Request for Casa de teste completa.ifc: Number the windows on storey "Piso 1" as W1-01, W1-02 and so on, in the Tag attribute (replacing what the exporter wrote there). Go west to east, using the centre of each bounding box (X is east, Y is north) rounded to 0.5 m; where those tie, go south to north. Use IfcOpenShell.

First a look at what the model holds.

```python
import ifcopenshell
import ifcopenshell.util.element
import ifcopenshell.util.placement

model = ifcopenshell.open("Casa de teste completa.ifc")
print(model.schema)
storey = next(s for s in model.by_type("IfcBuildingStorey") if s.Name == "Piso 1")
windows = [e for e in ifcopenshell.util.element.get_decomposition(storey) if e.is_a("IfcWindow")]
for e in sorted(windows, key=lambda e: e.id()):
    origin = ifcopenshell.util.placement.get_local_placement(e.ObjectPlacement)[:3, 3]
    print(e.id(), e.Tag, e.Name, origin.round(2) + 0.0, sep=" | ")
```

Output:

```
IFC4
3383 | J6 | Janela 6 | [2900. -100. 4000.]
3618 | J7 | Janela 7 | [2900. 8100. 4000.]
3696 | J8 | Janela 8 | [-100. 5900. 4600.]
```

```python
import ifcopenshell
import ifcopenshell.geom
import ifcopenshell.util.element
import ifcopenshell.util.shape

model = ifcopenshell.open("Casa de teste completa.ifc")
settings = ifcopenshell.geom.settings()
settings.set("use-world-coords", True)


def centre(element):
    shape = ifcopenshell.geom.create_shape(settings, element)
    return ifcopenshell.util.shape.get_bbox_centroid(shape.geometry)


storey = next(s for s in model.by_type("IfcBuildingStorey") if s.Name == "Piso 1")
windows = [e for e in ifcopenshell.util.element.get_decomposition(storey) if e.is_a("IfcWindow")]

# Insertion points can sit at a corner or the storey origin, so sort by the geometry (in metres).
centres = {e: centre(e) for e in windows}
windows.sort(key=lambda e: (round(centres[e][0] / 0.5), centres[e][1]))

for i, e in enumerate(windows, start=1):
    number = f"W1-{i:02d}"
    e.Tag = number
    print(e.id(), number)

model.write("Casa de teste completa-out.ifc")
```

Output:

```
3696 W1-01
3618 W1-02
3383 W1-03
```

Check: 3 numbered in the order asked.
